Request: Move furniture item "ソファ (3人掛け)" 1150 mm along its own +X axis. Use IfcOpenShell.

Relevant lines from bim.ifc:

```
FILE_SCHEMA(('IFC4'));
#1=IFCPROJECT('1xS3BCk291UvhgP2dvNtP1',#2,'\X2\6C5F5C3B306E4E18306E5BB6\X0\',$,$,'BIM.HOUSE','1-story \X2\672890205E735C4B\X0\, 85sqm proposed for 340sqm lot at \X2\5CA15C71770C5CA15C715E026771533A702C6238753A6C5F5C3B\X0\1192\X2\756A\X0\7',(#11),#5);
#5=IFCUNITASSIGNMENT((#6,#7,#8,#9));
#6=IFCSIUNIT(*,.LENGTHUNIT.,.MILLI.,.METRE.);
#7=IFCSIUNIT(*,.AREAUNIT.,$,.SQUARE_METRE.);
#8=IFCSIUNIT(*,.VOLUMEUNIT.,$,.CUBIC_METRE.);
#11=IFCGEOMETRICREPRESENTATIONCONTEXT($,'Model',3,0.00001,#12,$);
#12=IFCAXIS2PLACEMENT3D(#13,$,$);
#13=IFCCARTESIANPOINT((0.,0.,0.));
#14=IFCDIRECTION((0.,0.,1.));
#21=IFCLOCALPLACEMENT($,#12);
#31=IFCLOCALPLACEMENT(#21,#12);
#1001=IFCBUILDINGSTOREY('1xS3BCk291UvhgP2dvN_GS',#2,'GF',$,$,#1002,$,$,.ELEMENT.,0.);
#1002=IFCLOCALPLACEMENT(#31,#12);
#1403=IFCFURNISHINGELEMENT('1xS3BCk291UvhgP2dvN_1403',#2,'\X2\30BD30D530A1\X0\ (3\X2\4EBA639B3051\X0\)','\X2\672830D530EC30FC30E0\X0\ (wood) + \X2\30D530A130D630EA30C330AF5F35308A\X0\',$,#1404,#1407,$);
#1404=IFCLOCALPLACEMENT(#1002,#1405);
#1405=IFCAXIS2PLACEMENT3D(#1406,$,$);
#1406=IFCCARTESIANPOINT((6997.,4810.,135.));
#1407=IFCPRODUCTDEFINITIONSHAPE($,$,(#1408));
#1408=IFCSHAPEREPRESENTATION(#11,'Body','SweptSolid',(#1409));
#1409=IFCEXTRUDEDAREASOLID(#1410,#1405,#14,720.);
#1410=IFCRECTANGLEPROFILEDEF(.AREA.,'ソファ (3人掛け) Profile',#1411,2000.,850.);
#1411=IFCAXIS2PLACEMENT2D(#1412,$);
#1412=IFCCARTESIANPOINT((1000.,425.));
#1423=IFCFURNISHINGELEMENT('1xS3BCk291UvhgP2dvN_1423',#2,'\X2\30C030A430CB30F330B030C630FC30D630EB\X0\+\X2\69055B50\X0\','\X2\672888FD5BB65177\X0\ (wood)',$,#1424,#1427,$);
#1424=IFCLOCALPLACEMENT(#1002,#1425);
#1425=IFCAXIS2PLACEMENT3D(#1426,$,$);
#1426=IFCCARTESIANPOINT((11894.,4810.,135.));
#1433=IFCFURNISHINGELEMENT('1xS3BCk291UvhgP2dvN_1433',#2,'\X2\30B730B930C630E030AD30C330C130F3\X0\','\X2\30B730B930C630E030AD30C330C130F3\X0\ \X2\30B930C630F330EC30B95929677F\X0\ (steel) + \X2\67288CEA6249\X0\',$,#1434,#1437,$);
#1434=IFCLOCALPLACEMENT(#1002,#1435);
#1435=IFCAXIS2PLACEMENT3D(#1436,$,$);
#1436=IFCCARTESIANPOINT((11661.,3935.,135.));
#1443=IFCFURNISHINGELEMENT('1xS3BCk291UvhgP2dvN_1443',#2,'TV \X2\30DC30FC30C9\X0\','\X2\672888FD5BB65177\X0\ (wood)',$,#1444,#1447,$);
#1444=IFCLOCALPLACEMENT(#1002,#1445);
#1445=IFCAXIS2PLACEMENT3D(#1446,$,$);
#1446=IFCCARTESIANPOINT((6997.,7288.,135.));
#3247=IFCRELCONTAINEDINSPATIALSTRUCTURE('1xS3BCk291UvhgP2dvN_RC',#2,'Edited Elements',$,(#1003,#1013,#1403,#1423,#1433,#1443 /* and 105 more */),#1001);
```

```python
import ifcopenshell
import ifcopenshell.api.geometry
import ifcopenshell.util.placement
import ifcopenshell.util.unit

model = ifcopenshell.open("bim.ifc")
unit_scale = ifcopenshell.util.unit.calculate_unit_scale(model)

item = model.by_id(1403)
matrix = ifcopenshell.util.placement.get_local_placement(item.ObjectPlacement)
matrix[:3, 3] += matrix[:3, 0] * 1.15 / unit_scale
ifcopenshell.api.geometry.edit_object_placement(model, product=item, matrix=matrix, is_si=False)

print(ifcopenshell.util.placement.get_local_placement(item.ObjectPlacement).round(3) + 0.0)

model.write("bim_updated.ifc")
```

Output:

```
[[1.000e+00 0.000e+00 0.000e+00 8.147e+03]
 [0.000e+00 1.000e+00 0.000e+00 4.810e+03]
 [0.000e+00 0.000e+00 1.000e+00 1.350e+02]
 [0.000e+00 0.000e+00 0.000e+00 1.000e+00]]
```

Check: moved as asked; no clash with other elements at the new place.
